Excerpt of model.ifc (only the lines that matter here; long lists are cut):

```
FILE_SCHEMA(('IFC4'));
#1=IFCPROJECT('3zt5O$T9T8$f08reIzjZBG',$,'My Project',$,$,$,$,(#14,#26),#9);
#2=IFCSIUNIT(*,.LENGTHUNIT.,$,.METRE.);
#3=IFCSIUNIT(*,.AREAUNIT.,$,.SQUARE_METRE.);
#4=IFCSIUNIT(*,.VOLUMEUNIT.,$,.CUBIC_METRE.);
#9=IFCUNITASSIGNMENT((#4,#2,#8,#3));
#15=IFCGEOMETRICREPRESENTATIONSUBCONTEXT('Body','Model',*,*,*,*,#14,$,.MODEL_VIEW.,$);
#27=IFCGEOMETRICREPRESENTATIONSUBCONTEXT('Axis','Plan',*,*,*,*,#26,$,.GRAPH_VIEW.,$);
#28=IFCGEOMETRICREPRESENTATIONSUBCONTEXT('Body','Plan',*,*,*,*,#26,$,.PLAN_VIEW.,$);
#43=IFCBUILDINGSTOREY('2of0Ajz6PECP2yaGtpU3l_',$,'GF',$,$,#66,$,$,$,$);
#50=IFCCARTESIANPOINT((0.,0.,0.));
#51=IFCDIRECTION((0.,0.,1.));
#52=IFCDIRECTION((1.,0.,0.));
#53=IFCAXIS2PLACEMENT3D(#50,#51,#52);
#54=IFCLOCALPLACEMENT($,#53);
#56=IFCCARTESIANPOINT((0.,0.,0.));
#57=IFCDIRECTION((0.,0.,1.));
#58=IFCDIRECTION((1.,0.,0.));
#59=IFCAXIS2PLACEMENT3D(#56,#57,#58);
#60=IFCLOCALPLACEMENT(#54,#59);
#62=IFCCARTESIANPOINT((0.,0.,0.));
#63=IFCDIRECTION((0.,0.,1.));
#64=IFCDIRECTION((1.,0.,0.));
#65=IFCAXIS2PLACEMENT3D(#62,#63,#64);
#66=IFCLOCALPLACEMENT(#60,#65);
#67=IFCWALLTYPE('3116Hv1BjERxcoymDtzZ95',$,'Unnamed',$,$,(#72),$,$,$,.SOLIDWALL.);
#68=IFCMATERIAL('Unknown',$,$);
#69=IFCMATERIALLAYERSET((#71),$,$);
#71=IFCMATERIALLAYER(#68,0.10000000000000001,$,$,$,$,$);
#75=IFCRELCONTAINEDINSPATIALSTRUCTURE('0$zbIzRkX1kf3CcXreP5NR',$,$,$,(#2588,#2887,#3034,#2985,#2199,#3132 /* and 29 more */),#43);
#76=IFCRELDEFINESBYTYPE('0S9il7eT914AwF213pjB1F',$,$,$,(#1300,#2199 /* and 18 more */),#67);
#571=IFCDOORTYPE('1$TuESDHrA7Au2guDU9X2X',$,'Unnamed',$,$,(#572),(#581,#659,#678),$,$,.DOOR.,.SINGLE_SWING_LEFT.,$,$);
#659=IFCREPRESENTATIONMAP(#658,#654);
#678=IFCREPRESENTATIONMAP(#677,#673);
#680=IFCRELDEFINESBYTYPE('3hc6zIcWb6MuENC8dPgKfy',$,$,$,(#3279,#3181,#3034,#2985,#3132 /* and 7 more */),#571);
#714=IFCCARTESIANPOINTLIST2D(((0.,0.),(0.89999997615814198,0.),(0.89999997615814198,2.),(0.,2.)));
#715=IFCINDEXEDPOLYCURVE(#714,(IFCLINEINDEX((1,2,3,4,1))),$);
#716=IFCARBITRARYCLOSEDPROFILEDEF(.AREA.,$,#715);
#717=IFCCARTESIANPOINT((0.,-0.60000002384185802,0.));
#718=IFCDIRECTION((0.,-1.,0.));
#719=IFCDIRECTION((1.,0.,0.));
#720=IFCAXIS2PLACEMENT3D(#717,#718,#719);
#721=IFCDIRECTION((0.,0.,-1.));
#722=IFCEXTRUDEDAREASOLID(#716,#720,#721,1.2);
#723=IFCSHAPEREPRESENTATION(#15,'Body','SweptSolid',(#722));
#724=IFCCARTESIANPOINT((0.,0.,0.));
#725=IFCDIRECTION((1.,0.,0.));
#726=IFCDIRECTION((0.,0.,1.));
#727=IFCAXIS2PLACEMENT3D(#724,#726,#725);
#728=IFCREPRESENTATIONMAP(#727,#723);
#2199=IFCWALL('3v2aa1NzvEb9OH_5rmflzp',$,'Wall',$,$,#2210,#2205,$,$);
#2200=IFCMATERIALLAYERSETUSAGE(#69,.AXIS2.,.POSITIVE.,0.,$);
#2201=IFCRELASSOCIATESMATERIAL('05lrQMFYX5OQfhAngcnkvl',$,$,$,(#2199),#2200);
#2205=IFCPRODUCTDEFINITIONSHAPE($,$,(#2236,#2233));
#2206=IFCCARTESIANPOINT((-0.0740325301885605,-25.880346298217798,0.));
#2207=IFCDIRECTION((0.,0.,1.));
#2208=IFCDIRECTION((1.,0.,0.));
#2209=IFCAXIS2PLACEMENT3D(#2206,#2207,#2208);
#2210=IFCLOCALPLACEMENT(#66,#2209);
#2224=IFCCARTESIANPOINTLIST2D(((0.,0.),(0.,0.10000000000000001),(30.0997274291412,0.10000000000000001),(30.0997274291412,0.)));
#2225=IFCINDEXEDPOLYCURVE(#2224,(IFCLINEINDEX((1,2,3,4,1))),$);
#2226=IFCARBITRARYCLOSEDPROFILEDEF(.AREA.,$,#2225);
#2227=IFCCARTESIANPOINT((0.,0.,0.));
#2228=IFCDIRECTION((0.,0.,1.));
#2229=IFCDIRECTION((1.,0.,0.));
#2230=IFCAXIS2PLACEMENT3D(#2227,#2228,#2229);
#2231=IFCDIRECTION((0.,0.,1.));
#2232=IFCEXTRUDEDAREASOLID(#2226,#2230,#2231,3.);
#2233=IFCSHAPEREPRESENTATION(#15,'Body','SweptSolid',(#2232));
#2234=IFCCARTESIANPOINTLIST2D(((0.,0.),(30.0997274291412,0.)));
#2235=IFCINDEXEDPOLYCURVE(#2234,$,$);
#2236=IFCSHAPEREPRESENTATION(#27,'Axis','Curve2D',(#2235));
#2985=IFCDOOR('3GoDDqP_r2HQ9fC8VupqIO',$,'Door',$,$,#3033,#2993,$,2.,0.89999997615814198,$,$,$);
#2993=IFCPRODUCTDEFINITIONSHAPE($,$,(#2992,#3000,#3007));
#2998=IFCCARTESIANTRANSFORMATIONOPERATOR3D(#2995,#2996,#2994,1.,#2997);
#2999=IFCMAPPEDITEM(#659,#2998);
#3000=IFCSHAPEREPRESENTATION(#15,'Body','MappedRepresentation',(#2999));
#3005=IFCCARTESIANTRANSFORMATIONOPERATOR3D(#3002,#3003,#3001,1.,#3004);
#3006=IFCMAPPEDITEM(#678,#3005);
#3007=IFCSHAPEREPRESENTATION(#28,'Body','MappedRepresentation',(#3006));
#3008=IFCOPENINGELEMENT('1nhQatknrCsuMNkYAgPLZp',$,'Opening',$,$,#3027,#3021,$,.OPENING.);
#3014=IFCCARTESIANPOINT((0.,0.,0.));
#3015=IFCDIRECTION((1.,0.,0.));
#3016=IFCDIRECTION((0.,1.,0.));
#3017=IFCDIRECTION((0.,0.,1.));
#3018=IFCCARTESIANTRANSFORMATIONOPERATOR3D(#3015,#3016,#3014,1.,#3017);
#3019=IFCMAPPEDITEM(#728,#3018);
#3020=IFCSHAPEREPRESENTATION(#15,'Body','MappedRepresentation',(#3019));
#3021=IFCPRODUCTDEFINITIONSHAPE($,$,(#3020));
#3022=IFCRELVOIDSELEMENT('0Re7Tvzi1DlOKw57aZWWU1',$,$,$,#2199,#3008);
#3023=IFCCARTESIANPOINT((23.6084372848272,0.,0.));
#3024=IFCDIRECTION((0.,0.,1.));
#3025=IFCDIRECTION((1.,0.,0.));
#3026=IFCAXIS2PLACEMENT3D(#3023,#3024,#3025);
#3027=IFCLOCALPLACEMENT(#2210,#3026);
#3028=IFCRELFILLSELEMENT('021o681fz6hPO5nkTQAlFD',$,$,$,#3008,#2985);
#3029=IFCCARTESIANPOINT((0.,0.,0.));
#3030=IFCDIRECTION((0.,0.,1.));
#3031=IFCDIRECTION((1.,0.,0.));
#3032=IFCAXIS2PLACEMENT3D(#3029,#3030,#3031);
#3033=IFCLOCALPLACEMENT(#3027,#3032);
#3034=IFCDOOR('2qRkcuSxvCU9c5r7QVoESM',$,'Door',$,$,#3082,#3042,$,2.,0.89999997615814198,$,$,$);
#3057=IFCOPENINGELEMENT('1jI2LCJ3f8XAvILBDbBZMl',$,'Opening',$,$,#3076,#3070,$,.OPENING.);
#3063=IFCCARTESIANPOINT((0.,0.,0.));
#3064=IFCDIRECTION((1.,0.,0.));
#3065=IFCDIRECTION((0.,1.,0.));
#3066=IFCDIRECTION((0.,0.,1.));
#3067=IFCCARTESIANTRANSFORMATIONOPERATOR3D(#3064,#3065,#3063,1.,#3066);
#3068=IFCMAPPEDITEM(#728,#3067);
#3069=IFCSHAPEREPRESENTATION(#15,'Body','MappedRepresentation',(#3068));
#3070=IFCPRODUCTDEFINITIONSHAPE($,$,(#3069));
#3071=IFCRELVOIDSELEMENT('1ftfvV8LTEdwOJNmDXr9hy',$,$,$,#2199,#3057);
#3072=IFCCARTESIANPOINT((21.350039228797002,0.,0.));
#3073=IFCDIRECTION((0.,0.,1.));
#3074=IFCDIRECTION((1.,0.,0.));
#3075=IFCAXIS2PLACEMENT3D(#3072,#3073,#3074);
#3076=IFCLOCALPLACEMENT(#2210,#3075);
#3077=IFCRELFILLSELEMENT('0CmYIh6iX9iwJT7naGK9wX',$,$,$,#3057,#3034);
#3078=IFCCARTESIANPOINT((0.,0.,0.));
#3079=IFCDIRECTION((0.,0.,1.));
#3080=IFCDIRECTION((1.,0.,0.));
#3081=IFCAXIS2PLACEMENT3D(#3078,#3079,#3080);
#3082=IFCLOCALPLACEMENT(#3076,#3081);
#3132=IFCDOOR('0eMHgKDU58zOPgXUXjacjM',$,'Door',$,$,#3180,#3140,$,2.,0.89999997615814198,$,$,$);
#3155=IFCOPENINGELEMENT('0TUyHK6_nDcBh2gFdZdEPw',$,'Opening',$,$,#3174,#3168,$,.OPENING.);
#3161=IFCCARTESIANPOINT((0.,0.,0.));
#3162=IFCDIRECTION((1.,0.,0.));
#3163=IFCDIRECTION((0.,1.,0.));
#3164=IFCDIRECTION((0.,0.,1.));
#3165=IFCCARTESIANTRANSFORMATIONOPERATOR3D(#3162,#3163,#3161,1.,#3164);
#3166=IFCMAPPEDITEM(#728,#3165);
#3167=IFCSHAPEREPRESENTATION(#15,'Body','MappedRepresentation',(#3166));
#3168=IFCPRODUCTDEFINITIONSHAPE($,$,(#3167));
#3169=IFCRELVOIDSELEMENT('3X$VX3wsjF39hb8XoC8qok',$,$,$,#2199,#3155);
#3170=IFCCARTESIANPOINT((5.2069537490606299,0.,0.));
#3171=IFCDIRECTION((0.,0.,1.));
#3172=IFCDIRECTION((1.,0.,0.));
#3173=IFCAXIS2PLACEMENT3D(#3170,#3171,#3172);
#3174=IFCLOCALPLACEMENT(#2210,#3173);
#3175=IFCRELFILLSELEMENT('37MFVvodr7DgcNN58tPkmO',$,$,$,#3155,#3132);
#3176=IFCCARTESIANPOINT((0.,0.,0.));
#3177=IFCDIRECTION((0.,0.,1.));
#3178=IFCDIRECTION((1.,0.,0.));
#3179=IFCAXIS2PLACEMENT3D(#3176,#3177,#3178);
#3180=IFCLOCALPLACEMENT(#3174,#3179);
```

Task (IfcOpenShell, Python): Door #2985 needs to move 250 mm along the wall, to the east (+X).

```python
import ifcopenshell
import ifcopenshell.api.geometry
import ifcopenshell.util.placement
import ifcopenshell.util.unit

model = ifcopenshell.open("model.ifc")
unit_scale = ifcopenshell.util.unit.calculate_unit_scale(model)

door = model.by_id(2985)
opening = door.FillsVoids[0].RelatingOpeningElement
wall = opening.VoidsElements[0].RelatingBuildingElement

wall_matrix = ifcopenshell.util.placement.get_local_placement(wall.ObjectPlacement)
shift = wall_matrix[:3, 0] * 0.25 / unit_scale
before = ifcopenshell.util.placement.get_local_placement(door.ObjectPlacement)[:3, 3].copy()

# The door is placed relative to its opening, so it follows when the opening moves.
matrix = ifcopenshell.util.placement.get_local_placement(opening.ObjectPlacement)
matrix[:3, 3] += shift
ifcopenshell.api.geometry.edit_object_placement(
    model, product=opening, matrix=matrix, is_si=False, should_transform_children=True
)

after = ifcopenshell.util.placement.get_local_placement(door.ObjectPlacement)[:3, 3]
print("door moved by", (after - before).round(3) + 0.0)

model.write("model_edited.ifc")
```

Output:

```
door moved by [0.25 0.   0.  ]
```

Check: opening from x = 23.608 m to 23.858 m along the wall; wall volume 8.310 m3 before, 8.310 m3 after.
